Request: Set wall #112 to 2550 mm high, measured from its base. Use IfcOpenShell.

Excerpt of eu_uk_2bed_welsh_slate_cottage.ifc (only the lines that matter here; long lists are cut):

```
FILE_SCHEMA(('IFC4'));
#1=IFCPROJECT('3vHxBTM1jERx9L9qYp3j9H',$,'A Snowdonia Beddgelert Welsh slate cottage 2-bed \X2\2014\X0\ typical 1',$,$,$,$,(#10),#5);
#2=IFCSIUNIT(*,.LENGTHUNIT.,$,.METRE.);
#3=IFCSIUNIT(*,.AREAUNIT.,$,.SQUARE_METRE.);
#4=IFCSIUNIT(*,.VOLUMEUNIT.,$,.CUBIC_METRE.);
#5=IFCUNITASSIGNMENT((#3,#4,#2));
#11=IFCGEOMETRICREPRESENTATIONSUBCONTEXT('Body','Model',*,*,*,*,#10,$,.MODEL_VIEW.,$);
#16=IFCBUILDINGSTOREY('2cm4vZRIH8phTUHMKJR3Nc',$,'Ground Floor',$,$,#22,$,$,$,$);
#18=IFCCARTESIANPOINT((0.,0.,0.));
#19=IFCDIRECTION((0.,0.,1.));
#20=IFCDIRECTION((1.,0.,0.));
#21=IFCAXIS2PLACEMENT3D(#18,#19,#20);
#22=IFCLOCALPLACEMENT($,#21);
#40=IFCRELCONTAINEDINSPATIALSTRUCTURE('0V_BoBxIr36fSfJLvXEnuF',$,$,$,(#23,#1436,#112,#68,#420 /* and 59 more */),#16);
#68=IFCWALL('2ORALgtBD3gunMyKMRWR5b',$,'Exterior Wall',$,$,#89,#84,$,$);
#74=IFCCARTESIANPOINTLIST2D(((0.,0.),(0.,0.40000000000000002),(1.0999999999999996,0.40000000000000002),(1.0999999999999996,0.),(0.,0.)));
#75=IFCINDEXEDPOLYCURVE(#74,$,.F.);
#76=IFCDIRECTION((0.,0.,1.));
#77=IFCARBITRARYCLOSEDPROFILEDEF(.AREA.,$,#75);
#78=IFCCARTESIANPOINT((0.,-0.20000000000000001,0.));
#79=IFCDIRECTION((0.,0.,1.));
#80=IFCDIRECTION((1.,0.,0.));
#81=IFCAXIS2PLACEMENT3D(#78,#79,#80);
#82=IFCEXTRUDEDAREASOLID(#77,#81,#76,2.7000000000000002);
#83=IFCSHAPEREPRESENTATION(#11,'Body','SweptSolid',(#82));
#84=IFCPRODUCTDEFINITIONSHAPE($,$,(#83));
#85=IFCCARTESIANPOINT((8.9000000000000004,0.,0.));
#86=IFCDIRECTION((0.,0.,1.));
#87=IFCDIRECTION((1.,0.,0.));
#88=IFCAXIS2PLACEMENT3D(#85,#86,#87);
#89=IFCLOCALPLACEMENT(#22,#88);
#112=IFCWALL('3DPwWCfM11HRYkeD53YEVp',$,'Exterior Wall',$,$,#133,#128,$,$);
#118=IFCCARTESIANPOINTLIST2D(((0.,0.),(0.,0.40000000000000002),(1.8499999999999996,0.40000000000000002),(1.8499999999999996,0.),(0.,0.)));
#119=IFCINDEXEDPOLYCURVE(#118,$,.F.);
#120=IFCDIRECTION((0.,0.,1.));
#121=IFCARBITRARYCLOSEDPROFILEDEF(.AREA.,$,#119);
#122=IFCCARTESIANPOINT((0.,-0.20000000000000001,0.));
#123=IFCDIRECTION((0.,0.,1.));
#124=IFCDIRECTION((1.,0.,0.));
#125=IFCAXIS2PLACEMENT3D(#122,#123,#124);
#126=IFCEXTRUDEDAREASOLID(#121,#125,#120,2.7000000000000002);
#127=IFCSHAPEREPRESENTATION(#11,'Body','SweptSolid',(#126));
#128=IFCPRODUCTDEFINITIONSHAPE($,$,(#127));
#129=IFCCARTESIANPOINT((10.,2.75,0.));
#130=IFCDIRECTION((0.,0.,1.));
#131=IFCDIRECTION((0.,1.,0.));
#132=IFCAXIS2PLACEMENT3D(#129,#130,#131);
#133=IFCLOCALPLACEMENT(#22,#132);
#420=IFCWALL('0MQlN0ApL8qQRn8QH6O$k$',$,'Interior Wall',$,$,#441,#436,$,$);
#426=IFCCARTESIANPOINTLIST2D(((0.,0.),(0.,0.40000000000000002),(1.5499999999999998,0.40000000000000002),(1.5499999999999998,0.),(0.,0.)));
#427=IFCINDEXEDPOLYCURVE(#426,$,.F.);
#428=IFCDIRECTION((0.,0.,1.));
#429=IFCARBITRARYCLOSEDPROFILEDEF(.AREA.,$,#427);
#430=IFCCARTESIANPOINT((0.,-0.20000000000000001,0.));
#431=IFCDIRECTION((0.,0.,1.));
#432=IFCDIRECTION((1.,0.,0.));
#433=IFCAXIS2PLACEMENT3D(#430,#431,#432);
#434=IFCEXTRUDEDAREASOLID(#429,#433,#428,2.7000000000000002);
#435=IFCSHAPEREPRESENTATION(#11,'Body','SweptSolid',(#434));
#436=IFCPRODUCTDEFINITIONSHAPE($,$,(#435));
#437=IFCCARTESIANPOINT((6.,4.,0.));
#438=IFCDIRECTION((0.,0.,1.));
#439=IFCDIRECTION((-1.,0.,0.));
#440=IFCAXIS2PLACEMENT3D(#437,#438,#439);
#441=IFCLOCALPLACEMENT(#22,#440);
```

```python
import ifcopenshell
import ifcopenshell.geom
import ifcopenshell.util.representation
import ifcopenshell.util.shape
import ifcopenshell.util.unit

model = ifcopenshell.open("eu_uk_2bed_welsh_slate_cottage.ifc")
unit_scale = ifcopenshell.util.unit.calculate_unit_scale(model)
settings = ifcopenshell.geom.settings()


def volume(element):
    """Net volume in cubic metres, openings subtracted."""
    shape = ifcopenshell.geom.create_shape(settings, element)
    return ifcopenshell.util.shape.get_volume(shape.geometry)


wall = model.by_guid("3DPwWCfM11HRYkeD53YEVp")
before = volume(wall)

body = ifcopenshell.util.representation.get_representation(wall, "Model", "Body")
solid = body.Items[0]
old_height = solid.Depth
solid.Depth = 2.55 / unit_scale
after = volume(wall)

print(f"height {old_height:g} -> {solid.Depth:g}, volume {before:.3f} -> {after:.3f} m3")

model.write("eu_uk_2bed_welsh_slate_cottage-out.ifc")
```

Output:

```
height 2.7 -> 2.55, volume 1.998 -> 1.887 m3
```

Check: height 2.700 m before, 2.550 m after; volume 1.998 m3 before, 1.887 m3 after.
